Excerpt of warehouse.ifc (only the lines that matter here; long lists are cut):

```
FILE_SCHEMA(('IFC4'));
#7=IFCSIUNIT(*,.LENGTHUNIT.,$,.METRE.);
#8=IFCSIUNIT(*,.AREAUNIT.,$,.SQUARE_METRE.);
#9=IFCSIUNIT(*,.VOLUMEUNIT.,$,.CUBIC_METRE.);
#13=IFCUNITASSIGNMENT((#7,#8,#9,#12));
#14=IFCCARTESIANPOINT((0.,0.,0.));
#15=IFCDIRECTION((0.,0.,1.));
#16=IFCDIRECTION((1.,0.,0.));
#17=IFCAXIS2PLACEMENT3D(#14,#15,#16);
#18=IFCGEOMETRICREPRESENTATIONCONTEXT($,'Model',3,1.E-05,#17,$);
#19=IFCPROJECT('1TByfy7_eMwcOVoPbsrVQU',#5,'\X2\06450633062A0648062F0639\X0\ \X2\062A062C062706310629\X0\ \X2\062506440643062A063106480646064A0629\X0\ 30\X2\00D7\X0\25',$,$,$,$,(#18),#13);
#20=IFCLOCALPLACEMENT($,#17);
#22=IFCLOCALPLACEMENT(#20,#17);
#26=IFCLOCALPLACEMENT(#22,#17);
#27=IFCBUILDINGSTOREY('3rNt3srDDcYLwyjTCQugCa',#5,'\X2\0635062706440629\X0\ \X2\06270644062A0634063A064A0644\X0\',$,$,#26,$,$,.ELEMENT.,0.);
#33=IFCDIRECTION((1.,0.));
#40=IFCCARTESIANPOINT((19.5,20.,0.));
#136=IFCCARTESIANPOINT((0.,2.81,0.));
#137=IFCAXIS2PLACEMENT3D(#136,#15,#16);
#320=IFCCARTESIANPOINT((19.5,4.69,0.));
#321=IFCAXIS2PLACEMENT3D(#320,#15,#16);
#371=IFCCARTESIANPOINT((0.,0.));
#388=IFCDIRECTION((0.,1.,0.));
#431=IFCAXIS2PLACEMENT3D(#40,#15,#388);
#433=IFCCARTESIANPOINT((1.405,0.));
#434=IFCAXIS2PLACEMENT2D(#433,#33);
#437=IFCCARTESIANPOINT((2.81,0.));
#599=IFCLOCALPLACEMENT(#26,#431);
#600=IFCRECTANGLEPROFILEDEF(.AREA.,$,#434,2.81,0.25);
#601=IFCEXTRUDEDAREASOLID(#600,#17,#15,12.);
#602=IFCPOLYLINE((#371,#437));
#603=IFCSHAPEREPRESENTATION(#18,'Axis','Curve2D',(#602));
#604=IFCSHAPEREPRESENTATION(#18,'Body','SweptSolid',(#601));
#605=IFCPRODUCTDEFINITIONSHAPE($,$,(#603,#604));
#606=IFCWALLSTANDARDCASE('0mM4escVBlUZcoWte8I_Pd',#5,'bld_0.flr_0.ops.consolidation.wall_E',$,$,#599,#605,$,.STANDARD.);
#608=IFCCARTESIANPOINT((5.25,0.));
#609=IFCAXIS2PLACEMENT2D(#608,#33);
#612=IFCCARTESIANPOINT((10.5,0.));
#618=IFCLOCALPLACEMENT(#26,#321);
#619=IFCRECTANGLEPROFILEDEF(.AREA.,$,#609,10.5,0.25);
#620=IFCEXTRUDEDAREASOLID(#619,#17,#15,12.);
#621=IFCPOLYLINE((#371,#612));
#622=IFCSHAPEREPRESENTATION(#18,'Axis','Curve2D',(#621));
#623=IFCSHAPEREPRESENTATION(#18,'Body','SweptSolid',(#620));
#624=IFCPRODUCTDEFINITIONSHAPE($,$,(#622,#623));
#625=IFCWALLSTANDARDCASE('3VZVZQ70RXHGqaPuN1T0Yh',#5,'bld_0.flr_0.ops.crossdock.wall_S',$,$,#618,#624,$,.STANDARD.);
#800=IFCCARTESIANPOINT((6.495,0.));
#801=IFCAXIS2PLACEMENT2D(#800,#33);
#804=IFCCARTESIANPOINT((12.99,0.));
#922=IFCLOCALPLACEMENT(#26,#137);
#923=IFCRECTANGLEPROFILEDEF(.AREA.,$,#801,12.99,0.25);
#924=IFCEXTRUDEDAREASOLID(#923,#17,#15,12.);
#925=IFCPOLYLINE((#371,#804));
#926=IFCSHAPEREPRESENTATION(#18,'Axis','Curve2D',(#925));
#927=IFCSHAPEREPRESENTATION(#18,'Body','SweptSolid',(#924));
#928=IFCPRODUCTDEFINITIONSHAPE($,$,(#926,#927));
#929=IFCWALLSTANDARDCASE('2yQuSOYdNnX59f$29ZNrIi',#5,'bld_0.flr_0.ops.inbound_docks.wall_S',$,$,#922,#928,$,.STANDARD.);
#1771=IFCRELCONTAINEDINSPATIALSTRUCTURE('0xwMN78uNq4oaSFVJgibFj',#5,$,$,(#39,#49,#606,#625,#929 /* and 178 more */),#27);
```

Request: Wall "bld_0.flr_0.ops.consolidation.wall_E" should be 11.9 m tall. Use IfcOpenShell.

```python
import ifcopenshell
import ifcopenshell.geom
import ifcopenshell.util.shape
import ifcopenshell.util.unit

model = ifcopenshell.open("warehouse.ifc")
unit_scale = ifcopenshell.util.unit.calculate_unit_scale(model)
settings = ifcopenshell.geom.settings()


def volume(element):
    """Net volume in cubic metres, openings subtracted."""
    shape = ifcopenshell.geom.create_shape(settings, element)
    return ifcopenshell.util.shape.get_volume(shape.geometry)


wall = model.by_id(606)
before = volume(wall)

body = next(r for r in wall.Representation.Representations if r.RepresentationIdentifier == "Body")
solid = body.Items[0]
old_height = solid.Depth
solid.Depth = 11.9 / unit_scale
after = volume(wall)

print(f"height {old_height:g} -> {solid.Depth:g}, volume {before:.3f} -> {after:.3f} m3")

model.write("warehouse_rev.ifc")
```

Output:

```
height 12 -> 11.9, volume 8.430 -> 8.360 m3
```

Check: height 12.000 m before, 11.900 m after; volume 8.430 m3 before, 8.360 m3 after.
